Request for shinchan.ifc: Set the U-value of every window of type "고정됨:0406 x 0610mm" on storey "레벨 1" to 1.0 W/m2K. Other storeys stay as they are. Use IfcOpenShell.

First a look at what the model holds.

```python
import ifcopenshell
import ifcopenshell.util.element

model = ifcopenshell.open("shinchan.ifc")
print(model.schema)
storey = next(s for s in model.by_type("IfcBuildingStorey") if s.Name == "레벨 1")
windows = [e for e in ifcopenshell.util.element.get_decomposition(storey) if e.is_a("IfcWindow")]
seen = {}
for e in windows:
    element_type = ifcopenshell.util.element.get_type(e)
    key = (element_type.Name if element_type != e and element_type else None, ifcopenshell.util.element.get_pset(e, "Pset_WindowCommon", "ThermalTransmittance"))
    seen[key] = seen.get(key, 0) + 1
for (name, value), count in sorted(seen.items(), key=str):
    print(count, "x", name, "|", value)
```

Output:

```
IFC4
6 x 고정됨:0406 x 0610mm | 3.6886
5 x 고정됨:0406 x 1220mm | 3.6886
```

```python
import ifcopenshell
import ifcopenshell.api.pset
import ifcopenshell.util.element

model = ifcopenshell.open("shinchan.ifc")

storey = next(s for s in model.by_type("IfcBuildingStorey") if s.Name == "레벨 1")
windows = [e for e in ifcopenshell.util.element.get_decomposition(storey) if e.is_a("IfcWindow")]

count = 0
for e in windows:
    element_type = ifcopenshell.util.element.get_type(e)
    if element_type in (None, e) or element_type.Name != "고정됨:0406 x 0610mm":
        continue
    # add_pset returns the element's existing set when there is one.
    pset = ifcopenshell.api.pset.add_pset(model, product=e, name="Pset_WindowCommon")
    ifcopenshell.api.pset.edit_pset(model, pset=pset, properties={"ThermalTransmittance": 1.0})
    count += 1

print(count, "windows updated")

model.write("shinchan_v2.ifc")
```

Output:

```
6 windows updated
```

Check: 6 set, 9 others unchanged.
